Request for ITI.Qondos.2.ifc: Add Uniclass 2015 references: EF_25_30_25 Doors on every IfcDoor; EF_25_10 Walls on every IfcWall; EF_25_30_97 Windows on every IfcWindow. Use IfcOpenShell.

First a look at what the model holds.

```python
import ifcopenshell

model = ifcopenshell.open("ITI.Qondos.2.ifc")
print(model.schema)
print("classifications:", [c.Name for c in model.by_type("IfcClassification")])
for ifc_class in ("IfcDoor", "IfcRoof", "IfcStair", "IfcWall", "IfcWindow"):
    print(ifc_class, len(model.by_type(ifc_class)))
```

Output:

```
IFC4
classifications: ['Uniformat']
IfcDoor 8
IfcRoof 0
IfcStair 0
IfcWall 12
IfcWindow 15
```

```python
import ifcopenshell
import ifcopenshell.api.classification

model = ifcopenshell.open("ITI.Qondos.2.ifc")

system = ifcopenshell.api.classification.add_classification(model, classification="Uniclass 2015")

codes = {
    "IfcDoor": ("EF_25_30_25", "Doors"),
    "IfcWall": ("EF_25_10", "Walls"),
    "IfcWindow": ("EF_25_30_97", "Windows"),
}
for ifc_class, (code, name) in codes.items():
    products = model.by_type(ifc_class)
    ifcopenshell.api.classification.add_reference(
        model, products=products, classification=system, identification=code, name=name
    )
    print(code, len(products))

model.write("ITI.Qondos.2_rev.ifc")
```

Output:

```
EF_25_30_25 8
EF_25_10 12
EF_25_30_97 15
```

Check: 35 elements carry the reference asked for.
